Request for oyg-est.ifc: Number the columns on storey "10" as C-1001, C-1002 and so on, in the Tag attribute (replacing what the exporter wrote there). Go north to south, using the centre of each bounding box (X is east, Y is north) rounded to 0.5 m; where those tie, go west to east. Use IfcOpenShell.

First a look at what the model holds.

```python
import ifcopenshell
import ifcopenshell.util.element
import ifcopenshell.util.placement

model = ifcopenshell.open("oyg-est.ifc")
print(model.schema)
storey = next(s for s in model.by_type("IfcBuildingStorey") if s.Name == "10")
columns = [e for e in ifcopenshell.util.element.get_decomposition(storey) if e.is_a("IfcColumn")]
for e in sorted(columns, key=lambda e: e.id()):
    origin = ifcopenshell.util.placement.get_local_placement(e.ObjectPlacement)[:3, 3]
    print(e.id(), e.Tag, e.Name, origin.round(2) + 0.0, sep=" | ")
```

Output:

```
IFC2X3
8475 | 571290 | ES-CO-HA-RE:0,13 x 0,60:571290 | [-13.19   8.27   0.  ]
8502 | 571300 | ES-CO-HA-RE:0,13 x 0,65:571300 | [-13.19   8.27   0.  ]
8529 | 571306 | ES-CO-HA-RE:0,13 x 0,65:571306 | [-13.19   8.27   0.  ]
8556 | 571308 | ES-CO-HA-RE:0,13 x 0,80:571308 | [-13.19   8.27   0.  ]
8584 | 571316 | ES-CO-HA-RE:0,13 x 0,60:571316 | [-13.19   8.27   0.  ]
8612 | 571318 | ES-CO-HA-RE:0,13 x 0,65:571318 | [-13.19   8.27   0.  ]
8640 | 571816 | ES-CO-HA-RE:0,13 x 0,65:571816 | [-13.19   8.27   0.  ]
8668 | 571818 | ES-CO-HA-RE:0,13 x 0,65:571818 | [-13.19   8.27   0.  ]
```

```python
import ifcopenshell
import ifcopenshell.geom
import ifcopenshell.util.element
import ifcopenshell.util.shape

model = ifcopenshell.open("oyg-est.ifc")
settings = ifcopenshell.geom.settings()
settings.set("use-world-coords", True)


def centre(element):
    shape = ifcopenshell.geom.create_shape(settings, element)
    return ifcopenshell.util.shape.get_bbox_centroid(shape.geometry)


storey = next(s for s in model.by_type("IfcBuildingStorey") if s.Name == "10")
columns = [e for e in ifcopenshell.util.element.get_decomposition(storey) if e.is_a("IfcColumn")]

# Insertion points can sit at a corner or the storey origin, so sort by the geometry (in metres).
centres = {e: centre(e) for e in columns}
columns.sort(key=lambda e: (-round(centres[e][1] / 0.5), centres[e][0]))

for i, e in enumerate(columns, start=1):
    number = f"C-10{i:02d}"
    e.Tag = number
    print(e.id(), number)

model.write("oyg-est_v2.ifc")
```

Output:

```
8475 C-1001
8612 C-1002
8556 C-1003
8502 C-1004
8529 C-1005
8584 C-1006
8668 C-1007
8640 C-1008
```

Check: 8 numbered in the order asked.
